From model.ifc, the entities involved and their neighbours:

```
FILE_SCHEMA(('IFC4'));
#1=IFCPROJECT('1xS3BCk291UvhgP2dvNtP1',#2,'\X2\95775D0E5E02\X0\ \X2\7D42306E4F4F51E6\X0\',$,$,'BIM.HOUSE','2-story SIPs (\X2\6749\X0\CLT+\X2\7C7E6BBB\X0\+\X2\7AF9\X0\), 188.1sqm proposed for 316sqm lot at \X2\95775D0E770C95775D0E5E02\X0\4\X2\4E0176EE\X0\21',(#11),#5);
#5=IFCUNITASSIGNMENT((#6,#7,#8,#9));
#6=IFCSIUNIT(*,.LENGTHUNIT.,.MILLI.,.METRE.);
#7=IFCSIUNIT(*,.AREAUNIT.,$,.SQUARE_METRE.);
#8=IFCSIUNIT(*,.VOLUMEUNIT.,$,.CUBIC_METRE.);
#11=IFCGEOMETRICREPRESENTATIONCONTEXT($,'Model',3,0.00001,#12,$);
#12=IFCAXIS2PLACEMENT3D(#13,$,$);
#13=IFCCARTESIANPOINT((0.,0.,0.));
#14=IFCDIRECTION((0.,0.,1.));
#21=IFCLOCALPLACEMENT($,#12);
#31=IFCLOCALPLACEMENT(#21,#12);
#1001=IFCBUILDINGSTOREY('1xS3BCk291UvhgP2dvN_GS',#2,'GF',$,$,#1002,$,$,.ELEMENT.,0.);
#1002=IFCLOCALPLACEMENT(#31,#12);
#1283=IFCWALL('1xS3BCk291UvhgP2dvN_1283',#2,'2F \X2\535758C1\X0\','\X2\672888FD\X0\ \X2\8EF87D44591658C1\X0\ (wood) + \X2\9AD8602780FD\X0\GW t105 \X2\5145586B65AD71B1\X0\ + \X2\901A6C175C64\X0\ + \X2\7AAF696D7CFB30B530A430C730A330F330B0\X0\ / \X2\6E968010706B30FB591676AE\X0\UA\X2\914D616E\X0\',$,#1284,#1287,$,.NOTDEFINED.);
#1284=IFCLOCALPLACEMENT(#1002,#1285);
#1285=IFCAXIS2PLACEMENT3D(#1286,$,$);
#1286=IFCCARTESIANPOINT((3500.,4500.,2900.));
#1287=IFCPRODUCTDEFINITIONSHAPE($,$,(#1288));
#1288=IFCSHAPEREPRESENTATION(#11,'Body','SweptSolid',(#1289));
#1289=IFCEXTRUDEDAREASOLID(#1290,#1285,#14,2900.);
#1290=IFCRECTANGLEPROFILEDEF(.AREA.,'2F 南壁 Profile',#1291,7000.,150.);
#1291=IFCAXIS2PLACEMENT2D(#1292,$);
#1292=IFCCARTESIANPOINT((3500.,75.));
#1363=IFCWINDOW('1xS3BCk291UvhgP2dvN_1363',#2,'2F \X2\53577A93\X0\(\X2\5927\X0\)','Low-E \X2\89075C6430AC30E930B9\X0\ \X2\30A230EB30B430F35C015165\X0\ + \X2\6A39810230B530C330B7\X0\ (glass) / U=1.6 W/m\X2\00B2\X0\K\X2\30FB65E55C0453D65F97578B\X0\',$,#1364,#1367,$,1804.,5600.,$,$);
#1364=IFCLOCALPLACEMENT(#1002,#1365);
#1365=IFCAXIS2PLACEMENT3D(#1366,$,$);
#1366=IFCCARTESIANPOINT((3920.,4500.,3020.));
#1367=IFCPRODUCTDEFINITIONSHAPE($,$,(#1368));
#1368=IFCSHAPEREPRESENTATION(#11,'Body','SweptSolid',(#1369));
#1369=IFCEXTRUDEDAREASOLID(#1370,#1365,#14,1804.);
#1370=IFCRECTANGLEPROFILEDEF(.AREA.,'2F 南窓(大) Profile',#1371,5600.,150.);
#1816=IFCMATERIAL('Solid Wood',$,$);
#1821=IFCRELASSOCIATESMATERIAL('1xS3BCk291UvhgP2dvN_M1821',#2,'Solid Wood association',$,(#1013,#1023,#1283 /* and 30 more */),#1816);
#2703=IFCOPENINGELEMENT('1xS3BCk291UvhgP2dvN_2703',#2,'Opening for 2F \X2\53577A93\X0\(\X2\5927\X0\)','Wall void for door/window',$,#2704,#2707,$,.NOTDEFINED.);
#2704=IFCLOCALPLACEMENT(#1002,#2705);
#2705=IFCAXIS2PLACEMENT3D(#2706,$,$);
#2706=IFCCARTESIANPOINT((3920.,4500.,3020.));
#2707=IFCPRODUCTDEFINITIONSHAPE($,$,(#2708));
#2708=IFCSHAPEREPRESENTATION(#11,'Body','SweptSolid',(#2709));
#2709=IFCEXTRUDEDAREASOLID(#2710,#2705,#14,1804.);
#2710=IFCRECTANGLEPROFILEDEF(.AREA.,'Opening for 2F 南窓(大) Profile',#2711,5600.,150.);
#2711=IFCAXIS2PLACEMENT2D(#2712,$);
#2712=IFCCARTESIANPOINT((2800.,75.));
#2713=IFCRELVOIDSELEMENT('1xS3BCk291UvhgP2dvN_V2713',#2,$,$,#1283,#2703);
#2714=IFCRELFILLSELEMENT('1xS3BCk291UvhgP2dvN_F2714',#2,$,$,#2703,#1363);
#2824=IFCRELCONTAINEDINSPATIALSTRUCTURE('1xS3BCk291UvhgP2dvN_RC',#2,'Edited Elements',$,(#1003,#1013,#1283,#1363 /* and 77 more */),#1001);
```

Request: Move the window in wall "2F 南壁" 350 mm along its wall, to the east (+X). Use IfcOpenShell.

```python
import ifcopenshell
import ifcopenshell.api.geometry
import ifcopenshell.util.placement
import ifcopenshell.util.unit

model = ifcopenshell.open("model.ifc")
unit_scale = ifcopenshell.util.unit.calculate_unit_scale(model)

window = model.by_guid("1xS3BCk291UvhgP2dvN_1363")
opening = window.FillsVoids[0].RelatingOpeningElement
wall = opening.VoidsElements[0].RelatingBuildingElement

wall_matrix = ifcopenshell.util.placement.get_local_placement(wall.ObjectPlacement)
shift = wall_matrix[:3, 0] * 0.35 / unit_scale
before = ifcopenshell.util.placement.get_local_placement(window.ObjectPlacement)[:3, 3].copy()

# The window is not placed relative to its opening, so move both.
for product in (opening, window):
    matrix = ifcopenshell.util.placement.get_local_placement(product.ObjectPlacement)
    matrix[:3, 3] += shift
    ifcopenshell.api.geometry.edit_object_placement(model, product=product, matrix=matrix, is_si=False)

after = ifcopenshell.util.placement.get_local_placement(window.ObjectPlacement)[:3, 3]
print("window moved by", (after - before).round(3) + 0.0)

model.write("model_v2.ifc")
```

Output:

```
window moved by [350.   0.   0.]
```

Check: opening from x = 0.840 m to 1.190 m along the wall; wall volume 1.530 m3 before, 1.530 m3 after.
